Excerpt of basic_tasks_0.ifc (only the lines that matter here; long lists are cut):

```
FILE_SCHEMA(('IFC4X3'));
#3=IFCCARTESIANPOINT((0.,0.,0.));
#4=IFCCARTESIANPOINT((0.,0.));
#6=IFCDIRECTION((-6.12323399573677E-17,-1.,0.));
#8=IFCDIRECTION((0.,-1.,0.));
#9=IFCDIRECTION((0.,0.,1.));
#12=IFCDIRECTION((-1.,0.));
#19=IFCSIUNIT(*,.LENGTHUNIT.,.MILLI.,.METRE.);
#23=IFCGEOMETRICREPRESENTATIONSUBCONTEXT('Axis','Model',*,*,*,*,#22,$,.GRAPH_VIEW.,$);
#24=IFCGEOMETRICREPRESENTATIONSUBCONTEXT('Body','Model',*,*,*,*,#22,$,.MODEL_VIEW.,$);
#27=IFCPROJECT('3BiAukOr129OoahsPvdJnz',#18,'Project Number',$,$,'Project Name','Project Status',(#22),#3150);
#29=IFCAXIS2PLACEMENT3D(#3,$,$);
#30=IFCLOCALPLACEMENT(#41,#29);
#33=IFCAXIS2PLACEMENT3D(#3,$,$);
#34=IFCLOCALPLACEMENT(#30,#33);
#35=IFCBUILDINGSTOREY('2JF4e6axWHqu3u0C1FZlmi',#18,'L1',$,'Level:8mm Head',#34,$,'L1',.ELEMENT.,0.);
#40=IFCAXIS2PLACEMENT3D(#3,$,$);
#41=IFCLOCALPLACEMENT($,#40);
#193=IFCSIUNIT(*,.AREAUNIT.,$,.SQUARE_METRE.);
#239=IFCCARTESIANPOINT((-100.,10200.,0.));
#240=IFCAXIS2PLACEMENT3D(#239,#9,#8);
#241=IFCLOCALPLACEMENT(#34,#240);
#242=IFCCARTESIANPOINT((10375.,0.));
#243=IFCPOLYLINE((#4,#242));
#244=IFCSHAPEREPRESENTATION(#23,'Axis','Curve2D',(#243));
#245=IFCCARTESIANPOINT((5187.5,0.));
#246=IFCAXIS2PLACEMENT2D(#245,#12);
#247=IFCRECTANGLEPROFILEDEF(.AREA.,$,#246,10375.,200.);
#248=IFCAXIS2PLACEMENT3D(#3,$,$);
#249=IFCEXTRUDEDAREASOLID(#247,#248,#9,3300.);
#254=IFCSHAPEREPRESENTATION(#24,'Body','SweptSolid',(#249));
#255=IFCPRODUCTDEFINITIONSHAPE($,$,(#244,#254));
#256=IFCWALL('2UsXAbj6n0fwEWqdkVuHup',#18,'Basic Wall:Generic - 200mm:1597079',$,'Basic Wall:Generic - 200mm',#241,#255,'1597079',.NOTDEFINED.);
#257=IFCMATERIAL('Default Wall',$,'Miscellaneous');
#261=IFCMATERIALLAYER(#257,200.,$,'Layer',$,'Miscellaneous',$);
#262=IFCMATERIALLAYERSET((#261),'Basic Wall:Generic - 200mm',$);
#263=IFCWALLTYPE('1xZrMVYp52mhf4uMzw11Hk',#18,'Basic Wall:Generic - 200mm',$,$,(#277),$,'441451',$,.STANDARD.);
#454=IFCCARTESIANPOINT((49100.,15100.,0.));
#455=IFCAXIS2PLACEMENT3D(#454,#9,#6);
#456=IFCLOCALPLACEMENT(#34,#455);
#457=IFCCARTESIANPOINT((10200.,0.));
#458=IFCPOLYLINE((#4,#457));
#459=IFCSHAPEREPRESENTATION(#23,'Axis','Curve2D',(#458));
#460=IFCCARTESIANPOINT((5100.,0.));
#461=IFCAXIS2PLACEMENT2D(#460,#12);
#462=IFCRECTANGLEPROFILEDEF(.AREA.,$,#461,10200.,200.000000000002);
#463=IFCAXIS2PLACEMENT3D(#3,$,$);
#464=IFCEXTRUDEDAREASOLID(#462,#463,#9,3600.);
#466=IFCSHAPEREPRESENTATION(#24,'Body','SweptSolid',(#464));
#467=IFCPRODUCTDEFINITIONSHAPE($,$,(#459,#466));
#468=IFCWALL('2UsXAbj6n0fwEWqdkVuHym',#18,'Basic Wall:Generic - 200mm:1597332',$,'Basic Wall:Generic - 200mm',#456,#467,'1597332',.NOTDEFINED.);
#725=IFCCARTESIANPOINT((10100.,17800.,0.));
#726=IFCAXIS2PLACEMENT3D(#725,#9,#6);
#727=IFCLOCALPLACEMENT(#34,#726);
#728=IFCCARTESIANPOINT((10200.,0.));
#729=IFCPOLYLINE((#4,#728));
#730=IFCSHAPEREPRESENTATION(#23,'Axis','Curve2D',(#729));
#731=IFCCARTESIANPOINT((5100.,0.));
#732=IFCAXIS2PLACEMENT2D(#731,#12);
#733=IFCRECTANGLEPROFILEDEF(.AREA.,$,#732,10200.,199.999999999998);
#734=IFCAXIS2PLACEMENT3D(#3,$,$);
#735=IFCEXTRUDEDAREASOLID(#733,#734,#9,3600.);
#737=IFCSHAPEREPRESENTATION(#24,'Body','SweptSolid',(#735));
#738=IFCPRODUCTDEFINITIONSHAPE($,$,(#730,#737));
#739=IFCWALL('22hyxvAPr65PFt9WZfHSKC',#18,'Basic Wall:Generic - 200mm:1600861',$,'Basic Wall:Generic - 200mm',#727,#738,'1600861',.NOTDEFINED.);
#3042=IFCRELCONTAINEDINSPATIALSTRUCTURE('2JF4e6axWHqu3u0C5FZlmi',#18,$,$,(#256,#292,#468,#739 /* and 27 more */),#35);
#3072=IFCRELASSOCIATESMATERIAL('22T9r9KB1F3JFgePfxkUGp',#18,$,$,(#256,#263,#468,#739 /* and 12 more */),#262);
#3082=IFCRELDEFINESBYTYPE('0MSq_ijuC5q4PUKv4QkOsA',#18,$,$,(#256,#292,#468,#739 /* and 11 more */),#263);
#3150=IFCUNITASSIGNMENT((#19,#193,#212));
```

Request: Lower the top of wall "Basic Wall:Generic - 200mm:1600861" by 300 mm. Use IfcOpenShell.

```python
import ifcopenshell
import ifcopenshell.geom
import ifcopenshell.util.representation
import ifcopenshell.util.shape

model = ifcopenshell.open("basic_tasks_0.ifc")
settings = ifcopenshell.geom.settings()


def volume(element):
    """Net volume in cubic metres, openings subtracted."""
    shape = ifcopenshell.geom.create_shape(settings, element)
    return ifcopenshell.util.shape.get_volume(shape.geometry)


wall = model.by_guid("22hyxvAPr65PFt9WZfHSKC")
before = volume(wall)

body = ifcopenshell.util.representation.get_representation(wall, "Model", "Body")
solid = body.Items[0]
old_height = solid.Depth
solid.Depth -= 300.0
after = volume(wall)

print(f"height {old_height:g} -> {solid.Depth:g}, volume {before:.3f} -> {after:.3f} m3")

model.write("basic_tasks_0_edited.ifc")
```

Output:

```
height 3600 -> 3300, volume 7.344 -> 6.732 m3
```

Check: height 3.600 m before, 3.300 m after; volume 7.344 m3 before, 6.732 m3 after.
